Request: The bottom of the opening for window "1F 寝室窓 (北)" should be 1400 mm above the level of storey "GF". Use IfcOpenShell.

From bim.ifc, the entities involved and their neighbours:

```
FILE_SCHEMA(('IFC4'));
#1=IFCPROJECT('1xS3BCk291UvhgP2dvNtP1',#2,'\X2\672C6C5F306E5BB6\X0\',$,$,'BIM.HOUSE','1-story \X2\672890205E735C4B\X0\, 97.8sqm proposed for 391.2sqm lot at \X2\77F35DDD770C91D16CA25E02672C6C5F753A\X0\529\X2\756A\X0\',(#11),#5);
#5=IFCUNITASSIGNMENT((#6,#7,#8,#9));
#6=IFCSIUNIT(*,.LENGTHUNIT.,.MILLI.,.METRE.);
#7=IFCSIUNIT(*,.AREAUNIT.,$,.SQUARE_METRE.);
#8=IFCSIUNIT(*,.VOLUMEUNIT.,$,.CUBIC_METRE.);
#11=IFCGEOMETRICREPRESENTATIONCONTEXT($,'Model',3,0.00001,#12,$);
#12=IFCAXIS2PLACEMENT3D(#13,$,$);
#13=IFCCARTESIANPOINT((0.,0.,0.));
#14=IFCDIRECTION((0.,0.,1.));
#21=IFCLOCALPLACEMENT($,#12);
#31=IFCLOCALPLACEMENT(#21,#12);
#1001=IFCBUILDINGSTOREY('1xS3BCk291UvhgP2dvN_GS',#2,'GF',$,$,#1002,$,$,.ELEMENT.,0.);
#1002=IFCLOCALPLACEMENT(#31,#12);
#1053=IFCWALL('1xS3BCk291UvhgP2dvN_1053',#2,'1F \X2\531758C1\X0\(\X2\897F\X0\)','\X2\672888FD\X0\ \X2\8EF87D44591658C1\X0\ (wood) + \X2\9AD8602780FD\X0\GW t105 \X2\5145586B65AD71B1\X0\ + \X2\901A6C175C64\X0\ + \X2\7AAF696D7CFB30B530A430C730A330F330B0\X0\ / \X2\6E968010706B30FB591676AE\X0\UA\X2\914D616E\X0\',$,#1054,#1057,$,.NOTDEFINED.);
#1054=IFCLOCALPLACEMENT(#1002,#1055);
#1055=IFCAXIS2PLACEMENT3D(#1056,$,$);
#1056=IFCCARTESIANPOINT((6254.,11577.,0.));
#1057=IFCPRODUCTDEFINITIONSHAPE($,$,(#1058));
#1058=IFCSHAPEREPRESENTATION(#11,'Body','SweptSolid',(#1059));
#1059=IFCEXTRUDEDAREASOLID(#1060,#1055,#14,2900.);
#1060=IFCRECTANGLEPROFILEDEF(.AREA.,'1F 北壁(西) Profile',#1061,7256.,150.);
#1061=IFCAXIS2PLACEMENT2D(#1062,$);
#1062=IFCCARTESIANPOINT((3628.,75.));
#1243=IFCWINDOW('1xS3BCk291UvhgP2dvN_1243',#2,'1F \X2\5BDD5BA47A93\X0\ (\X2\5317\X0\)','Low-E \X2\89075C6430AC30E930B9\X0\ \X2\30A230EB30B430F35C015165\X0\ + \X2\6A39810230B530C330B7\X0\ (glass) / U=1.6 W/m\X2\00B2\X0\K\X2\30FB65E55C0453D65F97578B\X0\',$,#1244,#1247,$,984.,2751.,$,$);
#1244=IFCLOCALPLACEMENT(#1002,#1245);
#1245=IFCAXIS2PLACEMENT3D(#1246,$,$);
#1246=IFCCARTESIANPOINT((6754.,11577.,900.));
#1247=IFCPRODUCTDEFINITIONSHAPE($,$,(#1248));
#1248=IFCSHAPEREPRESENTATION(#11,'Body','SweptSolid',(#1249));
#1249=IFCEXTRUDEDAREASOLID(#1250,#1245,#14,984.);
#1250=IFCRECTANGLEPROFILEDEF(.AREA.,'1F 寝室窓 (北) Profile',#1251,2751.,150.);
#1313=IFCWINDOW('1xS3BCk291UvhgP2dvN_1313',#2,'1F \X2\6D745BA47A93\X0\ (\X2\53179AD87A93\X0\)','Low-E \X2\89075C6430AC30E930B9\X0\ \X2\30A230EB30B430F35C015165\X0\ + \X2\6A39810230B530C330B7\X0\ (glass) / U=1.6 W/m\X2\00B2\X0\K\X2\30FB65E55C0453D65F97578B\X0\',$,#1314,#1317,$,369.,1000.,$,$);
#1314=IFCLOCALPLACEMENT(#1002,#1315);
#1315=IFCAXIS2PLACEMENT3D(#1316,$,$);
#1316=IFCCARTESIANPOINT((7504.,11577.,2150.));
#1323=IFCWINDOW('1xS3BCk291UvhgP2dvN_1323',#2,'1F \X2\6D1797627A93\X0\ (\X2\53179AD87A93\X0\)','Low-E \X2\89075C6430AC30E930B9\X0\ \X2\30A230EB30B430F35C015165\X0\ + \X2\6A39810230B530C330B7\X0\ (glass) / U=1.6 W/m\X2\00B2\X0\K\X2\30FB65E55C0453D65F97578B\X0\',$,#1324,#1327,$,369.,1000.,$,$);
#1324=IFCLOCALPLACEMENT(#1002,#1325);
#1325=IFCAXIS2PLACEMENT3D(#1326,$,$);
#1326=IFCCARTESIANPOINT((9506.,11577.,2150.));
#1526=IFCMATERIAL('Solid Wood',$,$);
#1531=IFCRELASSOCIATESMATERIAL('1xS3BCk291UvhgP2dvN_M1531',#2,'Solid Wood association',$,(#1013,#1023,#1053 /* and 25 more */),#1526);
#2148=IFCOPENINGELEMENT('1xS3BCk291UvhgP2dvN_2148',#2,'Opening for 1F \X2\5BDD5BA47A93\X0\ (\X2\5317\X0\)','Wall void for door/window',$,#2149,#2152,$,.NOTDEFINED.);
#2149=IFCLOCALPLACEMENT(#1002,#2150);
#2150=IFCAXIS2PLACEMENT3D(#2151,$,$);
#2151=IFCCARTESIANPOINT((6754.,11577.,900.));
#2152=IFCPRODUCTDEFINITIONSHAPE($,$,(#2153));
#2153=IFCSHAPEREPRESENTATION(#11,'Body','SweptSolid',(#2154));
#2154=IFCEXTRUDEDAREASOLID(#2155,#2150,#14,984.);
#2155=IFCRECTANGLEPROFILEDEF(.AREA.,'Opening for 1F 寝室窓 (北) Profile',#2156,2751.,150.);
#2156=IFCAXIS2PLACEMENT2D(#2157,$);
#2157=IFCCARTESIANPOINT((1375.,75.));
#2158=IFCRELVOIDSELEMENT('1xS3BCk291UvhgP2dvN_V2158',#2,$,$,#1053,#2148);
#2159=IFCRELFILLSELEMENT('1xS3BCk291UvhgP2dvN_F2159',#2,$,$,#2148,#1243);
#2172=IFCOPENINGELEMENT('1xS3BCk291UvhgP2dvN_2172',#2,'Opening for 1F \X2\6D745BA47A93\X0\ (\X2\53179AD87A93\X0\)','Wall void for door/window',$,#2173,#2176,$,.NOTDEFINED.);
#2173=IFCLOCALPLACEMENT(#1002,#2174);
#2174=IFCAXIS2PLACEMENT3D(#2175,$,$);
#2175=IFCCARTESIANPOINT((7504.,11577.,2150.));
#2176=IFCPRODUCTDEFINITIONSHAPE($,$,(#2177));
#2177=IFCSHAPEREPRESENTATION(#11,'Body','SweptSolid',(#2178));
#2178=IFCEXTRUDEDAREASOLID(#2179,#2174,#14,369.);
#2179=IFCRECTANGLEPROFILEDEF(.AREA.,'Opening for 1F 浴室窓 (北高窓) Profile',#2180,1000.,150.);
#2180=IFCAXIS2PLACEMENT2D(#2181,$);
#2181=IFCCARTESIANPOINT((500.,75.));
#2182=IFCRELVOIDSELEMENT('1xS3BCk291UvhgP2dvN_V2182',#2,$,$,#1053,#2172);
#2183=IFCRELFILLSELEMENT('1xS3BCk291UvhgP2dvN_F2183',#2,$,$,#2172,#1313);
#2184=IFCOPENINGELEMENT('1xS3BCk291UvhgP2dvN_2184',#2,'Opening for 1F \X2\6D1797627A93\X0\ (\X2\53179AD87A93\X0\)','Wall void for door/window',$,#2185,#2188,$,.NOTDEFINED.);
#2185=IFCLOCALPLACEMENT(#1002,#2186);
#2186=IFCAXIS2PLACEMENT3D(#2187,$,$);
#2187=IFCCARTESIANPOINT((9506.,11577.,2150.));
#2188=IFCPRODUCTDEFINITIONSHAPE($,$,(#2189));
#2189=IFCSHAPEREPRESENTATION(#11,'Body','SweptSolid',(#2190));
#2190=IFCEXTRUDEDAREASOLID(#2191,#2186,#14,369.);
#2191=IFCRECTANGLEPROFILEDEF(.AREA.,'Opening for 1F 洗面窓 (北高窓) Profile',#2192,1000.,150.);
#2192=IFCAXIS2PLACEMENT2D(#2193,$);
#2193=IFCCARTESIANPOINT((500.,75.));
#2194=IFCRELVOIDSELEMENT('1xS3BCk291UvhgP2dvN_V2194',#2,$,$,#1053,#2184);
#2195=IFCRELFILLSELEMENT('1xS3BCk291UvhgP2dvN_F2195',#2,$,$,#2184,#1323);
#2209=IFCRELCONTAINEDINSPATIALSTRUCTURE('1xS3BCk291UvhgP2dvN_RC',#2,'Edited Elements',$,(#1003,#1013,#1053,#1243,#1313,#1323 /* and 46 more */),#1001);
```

```python
import numpy as np
import ifcopenshell
import ifcopenshell.api.geometry
import ifcopenshell.geom
import ifcopenshell.util.element
import ifcopenshell.util.placement
import ifcopenshell.util.shape
import ifcopenshell.util.unit

model = ifcopenshell.open("bim.ifc")
unit_scale = ifcopenshell.util.unit.calculate_unit_scale(model)

window = model.by_id(1243)
opening = window.FillsVoids[0].RelatingOpeningElement
storey = ifcopenshell.util.element.get_container(window, ifc_class="IfcBuildingStorey")
level = ifcopenshell.util.placement.get_local_placement(storey.ObjectPlacement)[2, 3]

# The opening's origin need not be at the sill, so measure its lowest point.
shape = ifcopenshell.geom.create_shape(ifcopenshell.geom.settings(), opening)
bottom = ifcopenshell.util.shape.get_shape_bottom_elevation(shape, shape.geometry) / unit_scale
dz = level + 1.4 / unit_scale - bottom

shift = np.array([0.0, 0.0, dz])
# The window is not placed relative to its opening, so move both.
for product in (opening, window):
    matrix = ifcopenshell.util.placement.get_local_placement(product.ObjectPlacement)
    matrix[:3, 3] += shift
    ifcopenshell.api.geometry.edit_object_placement(model, product=product, matrix=matrix, is_si=False)

print(f"moved by {dz * unit_scale:+.3f} m")

model.write("bim_rev.ifc")
```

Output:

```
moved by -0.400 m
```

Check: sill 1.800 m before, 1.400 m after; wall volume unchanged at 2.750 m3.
